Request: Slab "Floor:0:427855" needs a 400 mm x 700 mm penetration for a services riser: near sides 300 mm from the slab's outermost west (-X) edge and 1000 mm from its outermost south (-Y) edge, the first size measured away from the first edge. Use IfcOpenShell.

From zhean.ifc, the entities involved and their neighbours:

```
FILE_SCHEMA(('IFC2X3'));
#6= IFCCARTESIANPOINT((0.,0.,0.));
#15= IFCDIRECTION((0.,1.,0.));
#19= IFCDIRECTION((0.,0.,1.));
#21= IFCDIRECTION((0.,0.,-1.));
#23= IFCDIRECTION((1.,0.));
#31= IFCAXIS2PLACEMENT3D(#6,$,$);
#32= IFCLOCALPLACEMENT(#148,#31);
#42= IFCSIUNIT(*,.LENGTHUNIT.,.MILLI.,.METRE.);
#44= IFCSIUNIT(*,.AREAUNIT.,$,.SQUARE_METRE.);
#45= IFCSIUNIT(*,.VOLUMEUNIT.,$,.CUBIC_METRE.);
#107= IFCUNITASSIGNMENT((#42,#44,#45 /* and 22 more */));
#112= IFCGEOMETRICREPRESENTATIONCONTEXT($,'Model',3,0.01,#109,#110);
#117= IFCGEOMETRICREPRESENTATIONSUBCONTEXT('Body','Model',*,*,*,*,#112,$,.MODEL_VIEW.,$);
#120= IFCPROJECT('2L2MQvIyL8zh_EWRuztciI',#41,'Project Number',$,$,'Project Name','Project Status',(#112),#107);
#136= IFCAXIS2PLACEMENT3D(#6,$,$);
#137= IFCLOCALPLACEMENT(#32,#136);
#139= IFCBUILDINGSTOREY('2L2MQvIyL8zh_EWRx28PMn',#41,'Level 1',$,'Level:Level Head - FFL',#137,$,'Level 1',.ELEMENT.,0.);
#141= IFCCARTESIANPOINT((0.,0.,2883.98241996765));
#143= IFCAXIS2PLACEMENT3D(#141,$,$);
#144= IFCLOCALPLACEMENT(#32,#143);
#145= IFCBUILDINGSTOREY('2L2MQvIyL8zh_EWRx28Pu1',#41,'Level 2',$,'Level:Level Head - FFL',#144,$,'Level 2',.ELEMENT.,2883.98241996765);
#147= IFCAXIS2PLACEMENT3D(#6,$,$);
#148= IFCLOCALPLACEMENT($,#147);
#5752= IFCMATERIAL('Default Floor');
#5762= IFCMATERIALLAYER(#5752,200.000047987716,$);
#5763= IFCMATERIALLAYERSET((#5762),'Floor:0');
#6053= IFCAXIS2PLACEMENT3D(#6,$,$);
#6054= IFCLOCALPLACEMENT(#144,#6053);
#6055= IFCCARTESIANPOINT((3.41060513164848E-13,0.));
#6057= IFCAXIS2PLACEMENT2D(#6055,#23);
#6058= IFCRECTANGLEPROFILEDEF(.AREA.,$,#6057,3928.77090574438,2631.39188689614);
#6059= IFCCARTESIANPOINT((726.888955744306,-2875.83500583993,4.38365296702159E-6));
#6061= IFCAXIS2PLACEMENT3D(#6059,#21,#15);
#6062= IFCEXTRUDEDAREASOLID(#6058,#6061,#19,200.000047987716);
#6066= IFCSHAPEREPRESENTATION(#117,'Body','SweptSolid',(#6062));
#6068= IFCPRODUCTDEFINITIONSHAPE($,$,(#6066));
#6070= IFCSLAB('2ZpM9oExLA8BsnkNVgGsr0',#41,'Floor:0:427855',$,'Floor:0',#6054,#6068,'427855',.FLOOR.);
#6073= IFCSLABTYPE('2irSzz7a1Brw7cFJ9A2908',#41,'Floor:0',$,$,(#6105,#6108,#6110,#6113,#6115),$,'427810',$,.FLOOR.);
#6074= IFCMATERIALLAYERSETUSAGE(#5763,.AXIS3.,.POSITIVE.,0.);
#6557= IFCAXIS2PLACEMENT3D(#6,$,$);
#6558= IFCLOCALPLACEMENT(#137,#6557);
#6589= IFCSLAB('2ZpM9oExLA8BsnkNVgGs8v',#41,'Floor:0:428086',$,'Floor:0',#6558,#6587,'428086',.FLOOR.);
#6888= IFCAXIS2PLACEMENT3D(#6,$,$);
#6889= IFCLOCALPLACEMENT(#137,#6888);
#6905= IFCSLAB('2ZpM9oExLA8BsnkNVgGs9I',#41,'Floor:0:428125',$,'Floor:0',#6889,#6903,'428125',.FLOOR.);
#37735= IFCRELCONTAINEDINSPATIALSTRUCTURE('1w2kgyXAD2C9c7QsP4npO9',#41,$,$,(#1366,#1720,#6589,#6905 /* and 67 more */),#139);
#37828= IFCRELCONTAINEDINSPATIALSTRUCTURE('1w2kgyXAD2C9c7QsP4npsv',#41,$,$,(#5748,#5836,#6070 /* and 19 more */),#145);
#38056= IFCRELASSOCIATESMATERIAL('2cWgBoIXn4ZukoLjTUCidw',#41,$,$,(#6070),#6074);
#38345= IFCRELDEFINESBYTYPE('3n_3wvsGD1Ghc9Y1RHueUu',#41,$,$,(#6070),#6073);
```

```python
import numpy as np
import ifcopenshell
import ifcopenshell.api.feature
import ifcopenshell.api.geometry
import ifcopenshell.api.root
import ifcopenshell.geom
import ifcopenshell.util.placement
import ifcopenshell.util.representation
import ifcopenshell.util.shape
import ifcopenshell.util.unit

model = ifcopenshell.open("zhean.ifc")
unit_scale = ifcopenshell.util.unit.calculate_unit_scale(model)
settings = ifcopenshell.geom.settings()


def volume(element):
    """Net volume in cubic metres, openings subtracted."""
    shape = ifcopenshell.geom.create_shape(settings, element)
    return ifcopenshell.util.shape.get_volume(shape.geometry)


slab = model.by_guid("2ZpM9oExLA8BsnkNVgGsr0")
before = volume(slab)

# Extent in the slab's own axes, in metres. The edges named are its -X and -Y sides.
slab_shape = ifcopenshell.geom.create_shape(settings, slab)
vertices = ifcopenshell.util.shape.get_vertices(slab_shape.geometry)
x_min, y_min, bottom = vertices.min(axis=0)
top = vertices[:, 2].max()

opening = ifcopenshell.api.root.create_entity(model, ifc_class="IfcOpeningElement", name="Services riser opening")
context = ifcopenshell.util.representation.get_context(model, "Model", "Body", "MODEL_VIEW")
width, depth = 0.4, 0.7
outline = [(0.0, 0.0), (width, 0.0), (width, depth), (0.0, depth), (0.0, 0.0)]
# Overshoot both faces by 50 mm so the cut is clean.
shape = ifcopenshell.api.geometry.add_slab_representation(
    model, context=context, depth=top - bottom + 0.1, polyline=outline
)
ifcopenshell.api.geometry.assign_representation(model, product=opening, representation=shape)

matrix = ifcopenshell.util.placement.get_local_placement(slab.ObjectPlacement)
matrix[:, 3] = matrix @ np.append(np.array([x_min + 0.3, y_min + 1, bottom - 0.05]) / unit_scale, 1.0)
ifcopenshell.api.geometry.edit_object_placement(model, product=opening, matrix=matrix, is_si=False)
ifcopenshell.api.feature.add_feature(model, feature=opening, element=slab)

after = volume(slab)

print(f"slab volume {before:.3f} -> {after:.3f} m3")

model.write("zhean-out.ifc")
```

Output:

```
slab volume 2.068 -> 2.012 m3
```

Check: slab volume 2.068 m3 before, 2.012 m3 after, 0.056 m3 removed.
